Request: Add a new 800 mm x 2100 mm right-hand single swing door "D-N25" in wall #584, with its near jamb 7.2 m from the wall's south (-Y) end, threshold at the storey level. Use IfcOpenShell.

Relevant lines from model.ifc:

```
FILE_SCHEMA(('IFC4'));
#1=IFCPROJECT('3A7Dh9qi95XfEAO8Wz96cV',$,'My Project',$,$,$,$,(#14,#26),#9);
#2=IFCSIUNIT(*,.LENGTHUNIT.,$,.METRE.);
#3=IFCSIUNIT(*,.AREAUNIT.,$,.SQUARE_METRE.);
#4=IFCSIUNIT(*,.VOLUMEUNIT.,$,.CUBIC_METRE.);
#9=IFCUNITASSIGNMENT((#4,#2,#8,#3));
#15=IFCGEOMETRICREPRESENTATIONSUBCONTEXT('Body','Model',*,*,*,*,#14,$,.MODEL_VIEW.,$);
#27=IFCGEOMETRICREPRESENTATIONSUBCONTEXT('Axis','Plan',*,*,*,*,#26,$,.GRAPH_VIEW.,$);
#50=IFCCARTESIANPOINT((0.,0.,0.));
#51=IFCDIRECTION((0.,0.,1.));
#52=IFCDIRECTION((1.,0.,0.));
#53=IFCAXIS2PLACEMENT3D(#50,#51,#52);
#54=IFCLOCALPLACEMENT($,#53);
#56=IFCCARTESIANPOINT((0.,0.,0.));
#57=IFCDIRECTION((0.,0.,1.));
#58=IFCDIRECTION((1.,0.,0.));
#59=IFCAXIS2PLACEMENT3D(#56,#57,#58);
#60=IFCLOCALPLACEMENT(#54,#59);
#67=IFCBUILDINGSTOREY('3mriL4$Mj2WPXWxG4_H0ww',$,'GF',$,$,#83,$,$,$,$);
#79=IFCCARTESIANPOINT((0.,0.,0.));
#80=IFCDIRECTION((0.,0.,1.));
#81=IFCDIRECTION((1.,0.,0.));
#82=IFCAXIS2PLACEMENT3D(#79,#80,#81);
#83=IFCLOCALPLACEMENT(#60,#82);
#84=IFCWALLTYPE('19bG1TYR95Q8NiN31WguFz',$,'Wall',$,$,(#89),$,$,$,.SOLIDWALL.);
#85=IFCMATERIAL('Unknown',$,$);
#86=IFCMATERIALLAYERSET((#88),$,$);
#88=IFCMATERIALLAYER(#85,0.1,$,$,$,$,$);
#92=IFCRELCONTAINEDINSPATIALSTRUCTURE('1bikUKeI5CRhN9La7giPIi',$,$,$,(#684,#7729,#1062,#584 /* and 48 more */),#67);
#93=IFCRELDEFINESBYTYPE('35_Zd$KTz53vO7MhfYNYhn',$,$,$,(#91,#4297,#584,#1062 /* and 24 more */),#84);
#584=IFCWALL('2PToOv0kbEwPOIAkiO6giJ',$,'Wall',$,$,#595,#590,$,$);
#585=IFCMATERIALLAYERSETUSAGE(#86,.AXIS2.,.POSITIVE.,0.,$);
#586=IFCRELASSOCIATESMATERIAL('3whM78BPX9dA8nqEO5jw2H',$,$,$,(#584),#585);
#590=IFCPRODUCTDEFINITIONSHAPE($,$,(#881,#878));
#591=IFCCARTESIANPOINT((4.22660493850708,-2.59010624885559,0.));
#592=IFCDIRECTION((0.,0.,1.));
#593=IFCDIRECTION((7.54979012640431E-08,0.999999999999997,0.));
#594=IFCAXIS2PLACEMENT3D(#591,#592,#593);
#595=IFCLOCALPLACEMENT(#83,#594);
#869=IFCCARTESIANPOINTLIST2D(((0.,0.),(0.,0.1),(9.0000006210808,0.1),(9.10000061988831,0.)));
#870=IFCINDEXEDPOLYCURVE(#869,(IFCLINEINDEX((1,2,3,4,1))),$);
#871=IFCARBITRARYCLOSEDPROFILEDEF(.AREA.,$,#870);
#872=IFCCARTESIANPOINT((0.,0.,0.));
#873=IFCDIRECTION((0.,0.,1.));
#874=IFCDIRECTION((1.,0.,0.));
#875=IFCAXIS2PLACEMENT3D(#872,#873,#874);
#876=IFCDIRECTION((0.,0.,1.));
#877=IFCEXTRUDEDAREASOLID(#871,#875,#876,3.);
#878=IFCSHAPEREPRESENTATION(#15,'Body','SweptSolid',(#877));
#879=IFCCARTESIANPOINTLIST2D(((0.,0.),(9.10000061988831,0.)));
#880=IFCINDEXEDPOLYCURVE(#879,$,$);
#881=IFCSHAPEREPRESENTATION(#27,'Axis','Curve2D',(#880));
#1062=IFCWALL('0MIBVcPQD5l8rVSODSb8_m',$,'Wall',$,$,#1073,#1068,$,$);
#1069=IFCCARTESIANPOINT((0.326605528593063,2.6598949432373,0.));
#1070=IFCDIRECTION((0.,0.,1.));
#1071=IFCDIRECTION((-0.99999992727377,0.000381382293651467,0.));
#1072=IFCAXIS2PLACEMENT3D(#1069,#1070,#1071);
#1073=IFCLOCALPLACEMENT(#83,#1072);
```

```python
import numpy as np
import ifcopenshell
import ifcopenshell.api.feature
import ifcopenshell.api.geometry
import ifcopenshell.api.root
import ifcopenshell.api.spatial
import ifcopenshell.geom
import ifcopenshell.util.element
import ifcopenshell.util.placement
import ifcopenshell.util.representation
import ifcopenshell.util.shape
import ifcopenshell.util.unit

model = ifcopenshell.open("model.ifc")
unit_scale = ifcopenshell.util.unit.calculate_unit_scale(model)
settings = ifcopenshell.geom.settings()


def volume(element):
    """Net volume in cubic metres, openings subtracted."""
    shape = ifcopenshell.geom.create_shape(settings, element)
    return ifcopenshell.util.shape.get_volume(shape.geometry)


wall = model.by_id(584)
storey = ifcopenshell.util.element.get_container(wall, ifc_class="IfcBuildingStorey")
context = ifcopenshell.util.representation.get_context(model, "Model", "Body", "MODEL_VIEW")
before = volume(wall)

width, height, from_end, sill = 0.8, 2.1, 7.2, 0.0  # metres

# The wall runs along its own X axis, and the end named is its -X end.
wall_shape = ifcopenshell.geom.create_shape(settings, wall)
x, y, z = ifcopenshell.util.shape.get_vertices(wall_shape.geometry).T
start = x.min() + from_end
face, thickness = float(y.min()), float(y.max() - y.min())
wall_matrix = ifcopenshell.util.placement.get_local_placement(wall.ObjectPlacement)
level = ifcopenshell.util.placement.get_local_placement(storey.ObjectPlacement)[2, 3]


def in_wall(x, y):
    """Placement at x, y metres in the wall's axes, at sill height."""
    matrix = wall_matrix.copy()
    matrix[:, 3] = wall_matrix @ np.array([x / unit_scale, y / unit_scale, 0.0, 1.0])
    matrix[2, 3] = level + sill / unit_scale
    return matrix


# Opening: a box that overshoots both wall faces by 50 mm.
opening = ifcopenshell.api.root.create_entity(model, ifc_class="IfcOpeningElement", predefined_type="OPENING")
box = ifcopenshell.api.geometry.add_wall_representation(
    model, context=context, length=width, height=height, thickness=thickness + 0.1
)
ifcopenshell.api.geometry.assign_representation(model, product=opening, representation=box)
ifcopenshell.api.geometry.edit_object_placement(model, product=opening, matrix=in_wall(start, face - 0.05), is_si=False)
ifcopenshell.api.feature.add_feature(model, feature=opening, element=wall)

door = ifcopenshell.api.root.create_entity(model, ifc_class="IfcDoor", name="D-N25", predefined_type="DOOR")
door.OverallWidth, door.OverallHeight = width / unit_scale, height / unit_scale
door.OperationType = "SINGLE_SWING_RIGHT"
body = ifcopenshell.api.geometry.add_door_representation(
    model,
    context=context,
    overall_width=door.OverallWidth,
    overall_height=door.OverallHeight,
    operation_type="SINGLE_SWING_RIGHT",
    lining_properties={"LiningDepth": thickness / unit_scale, "ThresholdDepth": thickness / unit_scale},
)
ifcopenshell.api.geometry.assign_representation(model, product=door, representation=body)
ifcopenshell.api.spatial.assign_container(model, products=[door], relating_structure=storey)
ifcopenshell.api.feature.add_filling(model, opening=opening, element=door)

# The lining spans the wall, so the door starts at the wall face.
ifcopenshell.api.geometry.edit_object_placement(model, product=door, matrix=in_wall(start, face), is_si=False)

after = volume(wall)

print(f"wall volume {before:.3f} -> {after:.3f} m3")

model.write("model-out.ifc")
```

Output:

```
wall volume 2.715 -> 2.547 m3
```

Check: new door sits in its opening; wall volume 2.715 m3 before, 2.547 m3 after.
